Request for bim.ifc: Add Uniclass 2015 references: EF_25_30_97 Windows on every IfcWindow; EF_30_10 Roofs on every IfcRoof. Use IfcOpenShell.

First a look at what the model holds.

```python
import ifcopenshell

model = ifcopenshell.open("bim.ifc")
print(model.schema)
print("classifications:", [c.Name for c in model.by_type("IfcClassification")])
for ifc_class in ("IfcDoor", "IfcRoof", "IfcStair", "IfcWall", "IfcWindow"):
    print(ifc_class, len(model.by_type(ifc_class)))
```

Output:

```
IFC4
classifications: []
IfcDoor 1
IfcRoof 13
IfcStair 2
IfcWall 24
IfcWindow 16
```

```python
import ifcopenshell
import ifcopenshell.api.classification

model = ifcopenshell.open("bim.ifc")

system = ifcopenshell.api.classification.add_classification(model, classification="Uniclass 2015")

codes = {
    "IfcWindow": ("EF_25_30_97", "Windows"),
    "IfcRoof": ("EF_30_10", "Roofs"),
}
for ifc_class, (code, name) in codes.items():
    products = model.by_type(ifc_class)
    ifcopenshell.api.classification.add_reference(
        model, products=products, classification=system, identification=code, name=name
    )
    print(code, len(products))

model.write("bim_rev.ifc")
```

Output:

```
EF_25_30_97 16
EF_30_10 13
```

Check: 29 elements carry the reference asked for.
